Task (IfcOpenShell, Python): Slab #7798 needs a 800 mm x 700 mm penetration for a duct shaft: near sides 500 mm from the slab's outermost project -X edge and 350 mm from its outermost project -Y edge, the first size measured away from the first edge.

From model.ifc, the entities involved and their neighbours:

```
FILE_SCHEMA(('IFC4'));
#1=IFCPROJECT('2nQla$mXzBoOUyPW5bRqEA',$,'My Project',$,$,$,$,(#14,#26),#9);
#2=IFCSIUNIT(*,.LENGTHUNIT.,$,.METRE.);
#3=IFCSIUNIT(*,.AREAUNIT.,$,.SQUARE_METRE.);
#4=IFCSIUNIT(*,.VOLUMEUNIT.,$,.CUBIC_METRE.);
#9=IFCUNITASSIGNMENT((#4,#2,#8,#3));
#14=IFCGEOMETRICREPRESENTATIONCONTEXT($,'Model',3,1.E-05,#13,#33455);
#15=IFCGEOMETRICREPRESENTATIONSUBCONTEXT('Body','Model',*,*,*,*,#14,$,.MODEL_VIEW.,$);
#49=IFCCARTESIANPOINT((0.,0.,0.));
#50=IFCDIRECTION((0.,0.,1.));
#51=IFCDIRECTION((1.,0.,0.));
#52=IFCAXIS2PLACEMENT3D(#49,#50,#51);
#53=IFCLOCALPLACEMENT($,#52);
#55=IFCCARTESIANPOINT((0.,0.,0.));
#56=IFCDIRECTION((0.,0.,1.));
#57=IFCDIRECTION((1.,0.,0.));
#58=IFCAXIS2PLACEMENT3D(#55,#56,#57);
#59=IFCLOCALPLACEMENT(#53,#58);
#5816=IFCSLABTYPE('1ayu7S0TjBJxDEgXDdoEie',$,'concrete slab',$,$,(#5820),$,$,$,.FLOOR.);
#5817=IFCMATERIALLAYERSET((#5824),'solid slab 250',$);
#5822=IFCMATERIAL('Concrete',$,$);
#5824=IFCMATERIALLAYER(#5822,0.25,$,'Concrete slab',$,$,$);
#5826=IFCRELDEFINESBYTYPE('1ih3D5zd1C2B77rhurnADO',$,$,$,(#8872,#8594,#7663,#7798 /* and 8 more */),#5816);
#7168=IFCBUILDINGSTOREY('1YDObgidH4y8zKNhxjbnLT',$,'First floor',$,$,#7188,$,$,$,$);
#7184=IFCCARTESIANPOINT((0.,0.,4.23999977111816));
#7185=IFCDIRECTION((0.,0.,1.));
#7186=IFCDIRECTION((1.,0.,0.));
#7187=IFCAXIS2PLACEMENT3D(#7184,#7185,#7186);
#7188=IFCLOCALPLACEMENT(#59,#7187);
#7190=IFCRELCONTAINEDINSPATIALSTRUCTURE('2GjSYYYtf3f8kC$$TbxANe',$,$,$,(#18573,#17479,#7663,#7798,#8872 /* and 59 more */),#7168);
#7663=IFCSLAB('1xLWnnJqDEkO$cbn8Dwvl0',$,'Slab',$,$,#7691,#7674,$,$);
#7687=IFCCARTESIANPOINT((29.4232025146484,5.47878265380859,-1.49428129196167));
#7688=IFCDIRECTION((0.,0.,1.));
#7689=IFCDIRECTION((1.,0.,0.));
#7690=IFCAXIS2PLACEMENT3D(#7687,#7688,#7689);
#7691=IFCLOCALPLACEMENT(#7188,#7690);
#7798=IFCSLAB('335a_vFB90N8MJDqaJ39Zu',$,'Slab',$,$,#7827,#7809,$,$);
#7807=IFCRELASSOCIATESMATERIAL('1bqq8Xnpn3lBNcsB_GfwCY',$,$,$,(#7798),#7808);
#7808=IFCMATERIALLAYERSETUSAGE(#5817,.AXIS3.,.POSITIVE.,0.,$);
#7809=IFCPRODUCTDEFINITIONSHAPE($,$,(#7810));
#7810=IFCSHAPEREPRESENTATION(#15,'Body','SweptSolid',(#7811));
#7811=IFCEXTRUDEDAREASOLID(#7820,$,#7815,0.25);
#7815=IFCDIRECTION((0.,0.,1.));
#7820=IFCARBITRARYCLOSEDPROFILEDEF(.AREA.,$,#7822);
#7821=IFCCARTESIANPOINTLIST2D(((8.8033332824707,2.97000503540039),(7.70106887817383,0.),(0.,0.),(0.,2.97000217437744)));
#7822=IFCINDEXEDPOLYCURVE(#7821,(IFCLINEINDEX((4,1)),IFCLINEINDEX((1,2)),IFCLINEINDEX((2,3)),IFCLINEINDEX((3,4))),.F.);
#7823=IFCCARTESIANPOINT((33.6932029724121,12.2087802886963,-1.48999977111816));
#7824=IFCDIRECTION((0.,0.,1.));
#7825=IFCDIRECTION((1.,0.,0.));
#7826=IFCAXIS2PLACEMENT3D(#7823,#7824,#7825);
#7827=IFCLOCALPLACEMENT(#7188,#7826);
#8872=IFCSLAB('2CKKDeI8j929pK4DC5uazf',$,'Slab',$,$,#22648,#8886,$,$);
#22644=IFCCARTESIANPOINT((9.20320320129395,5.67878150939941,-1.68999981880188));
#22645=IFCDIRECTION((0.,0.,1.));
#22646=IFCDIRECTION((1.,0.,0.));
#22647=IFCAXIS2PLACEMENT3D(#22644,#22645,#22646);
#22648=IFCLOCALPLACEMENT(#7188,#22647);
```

```python
import numpy as np
import ifcopenshell
import ifcopenshell.api.feature
import ifcopenshell.api.geometry
import ifcopenshell.api.root
import ifcopenshell.geom
import ifcopenshell.util.placement
import ifcopenshell.util.representation
import ifcopenshell.util.shape
import ifcopenshell.util.unit

model = ifcopenshell.open("model.ifc")
unit_scale = ifcopenshell.util.unit.calculate_unit_scale(model)
settings = ifcopenshell.geom.settings()


def volume(element):
    """Net volume in cubic metres, openings subtracted."""
    shape = ifcopenshell.geom.create_shape(settings, element)
    return ifcopenshell.util.shape.get_volume(shape.geometry)


slab = model.by_guid("335a_vFB90N8MJDqaJ39Zu")
before = volume(slab)

# Extent in the slab's own axes, in metres. The edges named are its -X and -Y sides.
slab_shape = ifcopenshell.geom.create_shape(settings, slab)
vertices = ifcopenshell.util.shape.get_vertices(slab_shape.geometry)
x_min, y_min, bottom = vertices.min(axis=0)
top = vertices[:, 2].max()

opening = ifcopenshell.api.root.create_entity(model, ifc_class="IfcOpeningElement", name="Duct shaft opening", predefined_type="OPENING")
context = ifcopenshell.util.representation.get_context(model, "Model", "Body", "MODEL_VIEW")
width, depth = 0.8, 0.7
outline = [(0.0, 0.0), (width, 0.0), (width, depth), (0.0, depth), (0.0, 0.0)]
# Overshoot both faces by 50 mm so the cut is clean.
shape = ifcopenshell.api.geometry.add_slab_representation(
    model, context=context, depth=top - bottom + 0.1, polyline=outline
)
ifcopenshell.api.geometry.assign_representation(model, product=opening, representation=shape)

matrix = ifcopenshell.util.placement.get_local_placement(slab.ObjectPlacement)
matrix[:, 3] = matrix @ np.append(np.array([x_min + 0.5, y_min + 0.35, bottom - 0.05]) / unit_scale, 1.0)
ifcopenshell.api.geometry.edit_object_placement(model, product=opening, matrix=matrix, is_si=False)
ifcopenshell.api.feature.add_feature(model, feature=opening, element=slab)

after = volume(slab)

print(f"slab volume {before:.3f} -> {after:.3f} m3")

model.write("model-out.ifc")
```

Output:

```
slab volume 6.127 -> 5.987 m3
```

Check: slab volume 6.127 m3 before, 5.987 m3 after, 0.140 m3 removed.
